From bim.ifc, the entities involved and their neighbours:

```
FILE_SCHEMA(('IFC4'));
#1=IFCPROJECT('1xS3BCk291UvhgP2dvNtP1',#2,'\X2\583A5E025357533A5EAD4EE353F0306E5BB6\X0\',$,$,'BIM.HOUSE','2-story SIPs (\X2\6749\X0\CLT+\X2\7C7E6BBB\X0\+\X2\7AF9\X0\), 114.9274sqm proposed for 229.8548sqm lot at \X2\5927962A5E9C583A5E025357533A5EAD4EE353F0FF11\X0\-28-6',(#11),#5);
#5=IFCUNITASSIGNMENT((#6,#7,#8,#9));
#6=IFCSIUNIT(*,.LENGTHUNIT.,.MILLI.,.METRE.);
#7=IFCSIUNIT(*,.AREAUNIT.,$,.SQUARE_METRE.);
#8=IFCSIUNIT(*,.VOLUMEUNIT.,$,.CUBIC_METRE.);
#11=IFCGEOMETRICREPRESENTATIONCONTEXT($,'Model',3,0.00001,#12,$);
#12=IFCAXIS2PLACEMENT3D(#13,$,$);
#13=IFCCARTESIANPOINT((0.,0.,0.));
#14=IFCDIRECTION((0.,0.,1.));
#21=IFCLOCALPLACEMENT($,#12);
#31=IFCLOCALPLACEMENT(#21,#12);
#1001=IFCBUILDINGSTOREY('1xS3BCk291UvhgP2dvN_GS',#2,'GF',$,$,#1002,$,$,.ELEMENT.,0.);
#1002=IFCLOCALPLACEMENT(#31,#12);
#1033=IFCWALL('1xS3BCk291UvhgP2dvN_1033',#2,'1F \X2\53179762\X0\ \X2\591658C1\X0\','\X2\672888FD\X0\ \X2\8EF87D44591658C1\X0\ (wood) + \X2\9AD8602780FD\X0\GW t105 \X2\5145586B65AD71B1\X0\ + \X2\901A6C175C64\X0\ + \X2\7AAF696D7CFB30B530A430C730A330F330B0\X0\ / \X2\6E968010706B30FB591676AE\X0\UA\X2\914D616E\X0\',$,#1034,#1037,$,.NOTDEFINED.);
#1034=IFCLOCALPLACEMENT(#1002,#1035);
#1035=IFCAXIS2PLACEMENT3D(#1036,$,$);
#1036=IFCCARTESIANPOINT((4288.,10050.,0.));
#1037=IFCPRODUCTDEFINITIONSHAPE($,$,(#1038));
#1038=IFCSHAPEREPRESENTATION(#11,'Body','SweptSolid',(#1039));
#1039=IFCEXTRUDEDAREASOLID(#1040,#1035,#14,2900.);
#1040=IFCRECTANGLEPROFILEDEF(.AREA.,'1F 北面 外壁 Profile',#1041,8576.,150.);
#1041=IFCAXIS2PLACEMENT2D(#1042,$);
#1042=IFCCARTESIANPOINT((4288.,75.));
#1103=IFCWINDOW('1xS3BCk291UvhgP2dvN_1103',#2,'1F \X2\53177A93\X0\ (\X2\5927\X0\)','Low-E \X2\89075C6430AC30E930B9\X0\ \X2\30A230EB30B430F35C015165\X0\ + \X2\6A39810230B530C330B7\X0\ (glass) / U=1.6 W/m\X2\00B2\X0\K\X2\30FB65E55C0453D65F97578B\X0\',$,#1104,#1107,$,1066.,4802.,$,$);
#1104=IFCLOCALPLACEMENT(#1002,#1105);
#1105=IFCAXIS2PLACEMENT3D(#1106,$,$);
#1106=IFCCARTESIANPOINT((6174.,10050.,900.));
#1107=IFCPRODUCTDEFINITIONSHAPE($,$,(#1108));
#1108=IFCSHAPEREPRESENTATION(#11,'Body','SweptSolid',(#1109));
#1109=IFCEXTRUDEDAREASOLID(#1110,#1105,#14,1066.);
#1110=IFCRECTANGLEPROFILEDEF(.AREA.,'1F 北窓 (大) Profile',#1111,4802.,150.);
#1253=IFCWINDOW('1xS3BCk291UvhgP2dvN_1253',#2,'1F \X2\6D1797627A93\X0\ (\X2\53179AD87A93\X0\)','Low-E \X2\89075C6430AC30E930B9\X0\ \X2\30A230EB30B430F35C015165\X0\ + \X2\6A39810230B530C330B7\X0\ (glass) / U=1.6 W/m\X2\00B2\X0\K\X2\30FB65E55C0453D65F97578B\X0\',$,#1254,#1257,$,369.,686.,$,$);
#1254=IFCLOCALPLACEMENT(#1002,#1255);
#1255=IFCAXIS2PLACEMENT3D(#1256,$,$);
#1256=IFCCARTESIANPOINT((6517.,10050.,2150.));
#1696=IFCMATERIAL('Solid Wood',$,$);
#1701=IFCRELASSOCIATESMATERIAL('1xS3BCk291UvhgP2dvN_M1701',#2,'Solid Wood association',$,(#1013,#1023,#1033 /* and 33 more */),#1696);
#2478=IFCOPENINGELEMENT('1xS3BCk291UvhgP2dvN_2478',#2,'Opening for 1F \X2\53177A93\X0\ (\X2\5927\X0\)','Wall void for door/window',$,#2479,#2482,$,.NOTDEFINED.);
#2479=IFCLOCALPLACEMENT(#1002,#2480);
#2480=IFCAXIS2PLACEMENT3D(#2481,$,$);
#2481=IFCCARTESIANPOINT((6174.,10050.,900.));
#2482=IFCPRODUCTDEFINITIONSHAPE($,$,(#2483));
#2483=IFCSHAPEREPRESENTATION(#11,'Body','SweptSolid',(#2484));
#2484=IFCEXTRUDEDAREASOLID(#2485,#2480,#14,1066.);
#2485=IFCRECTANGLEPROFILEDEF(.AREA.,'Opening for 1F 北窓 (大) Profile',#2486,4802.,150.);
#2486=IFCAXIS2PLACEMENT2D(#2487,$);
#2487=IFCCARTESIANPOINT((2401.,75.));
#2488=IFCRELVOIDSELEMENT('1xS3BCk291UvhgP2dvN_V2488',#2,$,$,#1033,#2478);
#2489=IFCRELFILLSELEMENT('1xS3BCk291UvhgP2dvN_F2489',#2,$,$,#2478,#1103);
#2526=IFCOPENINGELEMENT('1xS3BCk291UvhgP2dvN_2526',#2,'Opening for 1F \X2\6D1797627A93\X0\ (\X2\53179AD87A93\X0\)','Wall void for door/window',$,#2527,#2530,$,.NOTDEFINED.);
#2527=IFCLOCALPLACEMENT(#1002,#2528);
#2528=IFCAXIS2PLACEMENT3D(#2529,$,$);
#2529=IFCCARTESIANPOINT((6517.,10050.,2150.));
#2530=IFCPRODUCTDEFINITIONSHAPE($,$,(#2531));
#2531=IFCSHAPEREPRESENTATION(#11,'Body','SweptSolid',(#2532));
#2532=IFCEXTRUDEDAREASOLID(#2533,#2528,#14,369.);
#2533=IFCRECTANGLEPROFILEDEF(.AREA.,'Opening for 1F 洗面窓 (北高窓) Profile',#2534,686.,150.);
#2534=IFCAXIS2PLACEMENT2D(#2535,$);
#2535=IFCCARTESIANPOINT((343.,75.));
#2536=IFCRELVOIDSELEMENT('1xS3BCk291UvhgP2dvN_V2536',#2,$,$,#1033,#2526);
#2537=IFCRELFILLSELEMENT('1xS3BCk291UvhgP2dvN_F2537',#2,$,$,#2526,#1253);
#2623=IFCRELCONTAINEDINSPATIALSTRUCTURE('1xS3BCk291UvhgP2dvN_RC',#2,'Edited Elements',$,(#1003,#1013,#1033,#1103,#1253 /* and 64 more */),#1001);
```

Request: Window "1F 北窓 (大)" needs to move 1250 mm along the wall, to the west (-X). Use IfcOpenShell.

```python
import ifcopenshell
import ifcopenshell.api.geometry
import ifcopenshell.util.placement

model = ifcopenshell.open("bim.ifc")

window = model.by_id(1103)
opening = window.FillsVoids[0].RelatingOpeningElement
wall = opening.VoidsElements[0].RelatingBuildingElement

wall_matrix = ifcopenshell.util.placement.get_local_placement(wall.ObjectPlacement)
shift = wall_matrix[:3, 0] * -1250.0
before = ifcopenshell.util.placement.get_local_placement(window.ObjectPlacement)[:3, 3].copy()

# The window is not placed relative to its opening, so move both.
for product in (opening, window):
    matrix = ifcopenshell.util.placement.get_local_placement(product.ObjectPlacement)
    matrix[:3, 3] += shift
    ifcopenshell.api.geometry.edit_object_placement(model, product=product, matrix=matrix, is_si=False)

after = ifcopenshell.util.placement.get_local_placement(window.ObjectPlacement)[:3, 3]
print("window moved by", (after - before).round(3) + 0.0)

model.write("bim_rev.ifc")
```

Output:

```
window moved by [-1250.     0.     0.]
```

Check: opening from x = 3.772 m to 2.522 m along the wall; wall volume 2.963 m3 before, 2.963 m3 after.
